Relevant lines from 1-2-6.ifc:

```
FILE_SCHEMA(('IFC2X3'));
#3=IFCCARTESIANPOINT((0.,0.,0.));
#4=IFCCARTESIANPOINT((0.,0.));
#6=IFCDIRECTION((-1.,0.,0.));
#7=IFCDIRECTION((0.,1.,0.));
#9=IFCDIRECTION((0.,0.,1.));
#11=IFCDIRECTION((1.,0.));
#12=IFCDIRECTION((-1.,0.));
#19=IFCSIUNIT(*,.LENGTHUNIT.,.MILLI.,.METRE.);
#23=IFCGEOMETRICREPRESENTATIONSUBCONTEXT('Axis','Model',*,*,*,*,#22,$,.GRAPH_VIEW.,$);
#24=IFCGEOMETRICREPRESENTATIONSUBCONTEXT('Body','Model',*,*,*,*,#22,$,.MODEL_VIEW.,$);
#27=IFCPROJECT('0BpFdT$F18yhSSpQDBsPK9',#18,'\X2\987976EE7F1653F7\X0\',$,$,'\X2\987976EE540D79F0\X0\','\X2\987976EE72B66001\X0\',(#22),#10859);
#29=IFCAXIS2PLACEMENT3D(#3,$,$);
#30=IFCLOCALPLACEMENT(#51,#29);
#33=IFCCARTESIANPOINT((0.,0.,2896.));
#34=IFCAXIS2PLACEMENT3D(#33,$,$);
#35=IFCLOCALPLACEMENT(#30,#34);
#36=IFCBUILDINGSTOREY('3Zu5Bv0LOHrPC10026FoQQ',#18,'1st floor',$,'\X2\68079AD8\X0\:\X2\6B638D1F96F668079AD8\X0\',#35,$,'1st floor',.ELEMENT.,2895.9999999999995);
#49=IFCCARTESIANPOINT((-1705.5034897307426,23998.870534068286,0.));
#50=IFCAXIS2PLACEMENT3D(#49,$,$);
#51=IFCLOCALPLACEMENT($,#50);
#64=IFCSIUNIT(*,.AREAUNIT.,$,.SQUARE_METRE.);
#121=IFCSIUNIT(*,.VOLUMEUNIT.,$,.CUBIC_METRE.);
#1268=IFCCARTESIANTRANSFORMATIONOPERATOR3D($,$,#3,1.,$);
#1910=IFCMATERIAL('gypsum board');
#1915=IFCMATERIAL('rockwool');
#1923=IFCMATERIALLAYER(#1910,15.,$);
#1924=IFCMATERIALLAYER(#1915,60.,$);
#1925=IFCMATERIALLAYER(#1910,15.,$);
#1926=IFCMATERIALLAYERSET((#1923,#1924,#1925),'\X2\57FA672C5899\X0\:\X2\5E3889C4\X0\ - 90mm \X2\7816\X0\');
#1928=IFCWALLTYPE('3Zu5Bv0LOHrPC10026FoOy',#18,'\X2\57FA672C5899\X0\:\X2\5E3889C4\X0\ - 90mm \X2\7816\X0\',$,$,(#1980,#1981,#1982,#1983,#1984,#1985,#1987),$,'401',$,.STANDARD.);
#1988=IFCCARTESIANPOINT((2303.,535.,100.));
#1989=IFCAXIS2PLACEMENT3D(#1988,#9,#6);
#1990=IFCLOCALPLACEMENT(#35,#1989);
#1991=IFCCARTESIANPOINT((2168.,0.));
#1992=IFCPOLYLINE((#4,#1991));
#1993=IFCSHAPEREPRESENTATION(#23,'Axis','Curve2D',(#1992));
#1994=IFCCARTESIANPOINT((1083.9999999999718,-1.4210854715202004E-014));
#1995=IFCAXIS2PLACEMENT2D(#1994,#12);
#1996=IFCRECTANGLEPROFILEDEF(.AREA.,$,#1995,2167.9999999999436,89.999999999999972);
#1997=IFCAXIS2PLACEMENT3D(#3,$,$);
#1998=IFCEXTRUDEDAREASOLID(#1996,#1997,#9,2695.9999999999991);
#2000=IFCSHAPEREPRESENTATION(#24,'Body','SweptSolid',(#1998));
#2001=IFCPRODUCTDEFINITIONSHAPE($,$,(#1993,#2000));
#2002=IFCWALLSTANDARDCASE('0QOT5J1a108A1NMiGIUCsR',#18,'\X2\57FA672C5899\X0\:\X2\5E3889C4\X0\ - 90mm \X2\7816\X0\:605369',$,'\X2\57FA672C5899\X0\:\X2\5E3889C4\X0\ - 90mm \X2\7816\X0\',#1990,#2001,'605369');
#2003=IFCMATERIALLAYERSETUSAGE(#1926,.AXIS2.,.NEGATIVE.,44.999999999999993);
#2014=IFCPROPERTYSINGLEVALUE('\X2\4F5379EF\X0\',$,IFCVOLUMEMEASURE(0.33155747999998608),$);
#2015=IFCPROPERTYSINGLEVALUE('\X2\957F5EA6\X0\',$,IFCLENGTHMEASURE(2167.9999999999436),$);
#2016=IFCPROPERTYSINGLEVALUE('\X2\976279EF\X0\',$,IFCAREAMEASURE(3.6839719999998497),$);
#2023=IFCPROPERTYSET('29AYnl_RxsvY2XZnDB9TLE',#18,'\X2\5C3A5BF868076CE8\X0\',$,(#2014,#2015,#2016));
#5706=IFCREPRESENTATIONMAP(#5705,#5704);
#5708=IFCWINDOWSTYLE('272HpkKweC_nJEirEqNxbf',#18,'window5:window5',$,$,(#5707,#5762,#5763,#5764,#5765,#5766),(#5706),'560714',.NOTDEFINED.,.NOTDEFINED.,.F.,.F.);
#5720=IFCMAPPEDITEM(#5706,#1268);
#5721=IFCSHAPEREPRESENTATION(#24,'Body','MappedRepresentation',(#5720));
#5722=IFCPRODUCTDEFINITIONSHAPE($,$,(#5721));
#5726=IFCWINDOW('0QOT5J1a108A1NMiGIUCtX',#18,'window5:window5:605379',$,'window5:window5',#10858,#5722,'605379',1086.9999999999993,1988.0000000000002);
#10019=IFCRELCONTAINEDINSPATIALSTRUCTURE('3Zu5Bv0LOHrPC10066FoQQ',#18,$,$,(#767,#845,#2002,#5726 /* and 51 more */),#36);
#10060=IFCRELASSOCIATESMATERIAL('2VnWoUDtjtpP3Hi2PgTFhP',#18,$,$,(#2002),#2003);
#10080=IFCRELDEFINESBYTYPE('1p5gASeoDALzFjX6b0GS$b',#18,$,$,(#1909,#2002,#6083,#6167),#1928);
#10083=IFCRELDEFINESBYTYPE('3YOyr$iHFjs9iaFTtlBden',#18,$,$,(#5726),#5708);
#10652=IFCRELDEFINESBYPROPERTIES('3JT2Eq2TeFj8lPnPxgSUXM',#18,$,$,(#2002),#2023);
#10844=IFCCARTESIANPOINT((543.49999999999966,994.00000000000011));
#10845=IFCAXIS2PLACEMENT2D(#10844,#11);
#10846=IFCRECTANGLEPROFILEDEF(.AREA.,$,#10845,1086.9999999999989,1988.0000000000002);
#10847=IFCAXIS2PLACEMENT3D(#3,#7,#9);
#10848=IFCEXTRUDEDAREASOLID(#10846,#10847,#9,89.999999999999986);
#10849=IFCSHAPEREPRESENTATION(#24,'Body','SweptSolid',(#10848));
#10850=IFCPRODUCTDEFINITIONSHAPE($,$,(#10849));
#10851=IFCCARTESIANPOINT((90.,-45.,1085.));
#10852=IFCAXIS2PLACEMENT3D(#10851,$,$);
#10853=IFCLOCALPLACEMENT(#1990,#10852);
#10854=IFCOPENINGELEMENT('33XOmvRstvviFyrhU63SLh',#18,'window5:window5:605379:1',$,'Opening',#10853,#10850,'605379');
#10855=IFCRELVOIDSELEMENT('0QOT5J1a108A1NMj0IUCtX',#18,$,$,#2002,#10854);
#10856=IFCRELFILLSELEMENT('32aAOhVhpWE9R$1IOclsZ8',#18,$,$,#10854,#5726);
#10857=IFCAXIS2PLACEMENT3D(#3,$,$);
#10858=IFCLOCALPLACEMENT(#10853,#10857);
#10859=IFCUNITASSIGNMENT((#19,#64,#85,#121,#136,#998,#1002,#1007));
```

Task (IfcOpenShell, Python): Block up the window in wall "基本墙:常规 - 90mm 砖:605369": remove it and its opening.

```python
import ifcopenshell
import ifcopenshell.api.feature
import ifcopenshell.api.pset
import ifcopenshell.api.root
import ifcopenshell.geom
import ifcopenshell.util.element
import ifcopenshell.util.shape
import ifcopenshell.util.unit

model = ifcopenshell.open("1-2-6.ifc")
area_scale = ifcopenshell.util.unit.calculate_unit_scale(model, "AREAUNIT")
volume_scale = ifcopenshell.util.unit.calculate_unit_scale(model, "VOLUMEUNIT")
settings = ifcopenshell.geom.settings()


def volume(element):
    """Net volume in cubic metres, openings subtracted."""
    shape = ifcopenshell.geom.create_shape(settings, element)
    return ifcopenshell.util.shape.get_volume(shape.geometry)


window = model.by_id(5726)
opening = window.FillsVoids[0].RelatingOpeningElement
wall = opening.VoidsElements[0].RelatingBuildingElement
before = volume(wall)

ifcopenshell.api.root.remove_product(model, product=window)
ifcopenshell.api.feature.remove_feature(model, feature=opening)

after = volume(wall)
thickness = 0.09  # wall thickness in metres

# Update the wall's stored quantities.
pset = model.by_id(ifcopenshell.util.element.get_pset(wall, "尺寸标注", should_inherit=False)["id"])
ifcopenshell.api.pset.edit_pset(model, pset=pset, properties={
    "体积": model.create_entity("IfcVolumeMeasure", after / volume_scale),
    "面积": model.create_entity("IfcAreaMeasure", after / thickness / area_scale),
})

print(f"wall volume {before:.3f} -> {after:.3f} m3")

model.write("1-2-6_edited.ifc")
```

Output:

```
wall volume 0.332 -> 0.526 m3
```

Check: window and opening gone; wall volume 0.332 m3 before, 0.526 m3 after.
